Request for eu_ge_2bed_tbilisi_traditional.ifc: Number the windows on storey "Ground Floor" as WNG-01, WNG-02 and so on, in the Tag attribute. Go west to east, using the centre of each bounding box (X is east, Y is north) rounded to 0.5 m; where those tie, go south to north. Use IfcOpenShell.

First a look at what the model holds.

```python
import ifcopenshell
import ifcopenshell.util.element
import ifcopenshell.util.placement

model = ifcopenshell.open("eu_ge_2bed_tbilisi_traditional.ifc")
print(model.schema)
storey = next(s for s in model.by_type("IfcBuildingStorey") if s.Name == "Ground Floor")
windows = [e for e in ifcopenshell.util.element.get_decomposition(storey) if e.is_a("IfcWindow")]
for e in sorted(windows, key=lambda e: e.id()):
    origin = ifcopenshell.util.placement.get_local_placement(e.ObjectPlacement)[:3, 3]
    print(e.id(), e.Tag, e.Name, origin.round(2) + 0.0, sep=" | ")
```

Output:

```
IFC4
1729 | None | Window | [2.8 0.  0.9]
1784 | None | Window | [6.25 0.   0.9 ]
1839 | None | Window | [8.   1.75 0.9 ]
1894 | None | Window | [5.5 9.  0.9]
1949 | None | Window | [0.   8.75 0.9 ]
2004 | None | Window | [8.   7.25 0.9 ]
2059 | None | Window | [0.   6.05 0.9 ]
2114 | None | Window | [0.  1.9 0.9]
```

```python
import ifcopenshell
import ifcopenshell.geom
import ifcopenshell.util.element
import ifcopenshell.util.shape

model = ifcopenshell.open("eu_ge_2bed_tbilisi_traditional.ifc")
settings = ifcopenshell.geom.settings()
settings.set("use-world-coords", True)


def centre(element):
    shape = ifcopenshell.geom.create_shape(settings, element)
    return ifcopenshell.util.shape.get_bbox_centroid(shape.geometry)


storey = next(s for s in model.by_type("IfcBuildingStorey") if s.Name == "Ground Floor")
windows = [e for e in ifcopenshell.util.element.get_decomposition(storey) if e.is_a("IfcWindow")]

# Insertion points can sit at a corner or the storey origin, so sort by the geometry (in metres).
centres = {e: centre(e) for e in windows}
windows.sort(key=lambda e: (round(centres[e][0] / 0.5), centres[e][1]))

for i, e in enumerate(windows, start=1):
    number = f"WNG-{i:02d}"
    e.Tag = number
    print(e.id(), number)

model.write("eu_ge_2bed_tbilisi_traditional_edited.ifc")
```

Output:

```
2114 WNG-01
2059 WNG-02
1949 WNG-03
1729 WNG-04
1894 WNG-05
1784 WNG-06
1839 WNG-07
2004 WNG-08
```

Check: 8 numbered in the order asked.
